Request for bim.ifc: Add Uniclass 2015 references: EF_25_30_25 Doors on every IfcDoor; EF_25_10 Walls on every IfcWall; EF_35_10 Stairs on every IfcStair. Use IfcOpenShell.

First a look at what the model holds.

```python
import ifcopenshell

model = ifcopenshell.open("bim.ifc")
print(model.schema)
print("classifications:", [c.Name for c in model.by_type("IfcClassification")])
for ifc_class in ("IfcDoor", "IfcRoof", "IfcStair", "IfcWall", "IfcWindow"):
    print(ifc_class, len(model.by_type(ifc_class)))
```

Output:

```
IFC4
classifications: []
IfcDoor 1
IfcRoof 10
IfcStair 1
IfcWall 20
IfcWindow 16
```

```python
import ifcopenshell
import ifcopenshell.api.classification

model = ifcopenshell.open("bim.ifc")

system = ifcopenshell.api.classification.add_classification(model, classification="Uniclass 2015")

codes = {
    "IfcDoor": ("EF_25_30_25", "Doors"),
    "IfcWall": ("EF_25_10", "Walls"),
    "IfcStair": ("EF_35_10", "Stairs"),
}
for ifc_class, (code, name) in codes.items():
    products = model.by_type(ifc_class)
    ifcopenshell.api.classification.add_reference(
        model, products=products, classification=system, identification=code, name=name
    )
    print(code, len(products))

model.write("bim_edited.ifc")
```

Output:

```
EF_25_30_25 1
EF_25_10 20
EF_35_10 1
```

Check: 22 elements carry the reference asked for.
